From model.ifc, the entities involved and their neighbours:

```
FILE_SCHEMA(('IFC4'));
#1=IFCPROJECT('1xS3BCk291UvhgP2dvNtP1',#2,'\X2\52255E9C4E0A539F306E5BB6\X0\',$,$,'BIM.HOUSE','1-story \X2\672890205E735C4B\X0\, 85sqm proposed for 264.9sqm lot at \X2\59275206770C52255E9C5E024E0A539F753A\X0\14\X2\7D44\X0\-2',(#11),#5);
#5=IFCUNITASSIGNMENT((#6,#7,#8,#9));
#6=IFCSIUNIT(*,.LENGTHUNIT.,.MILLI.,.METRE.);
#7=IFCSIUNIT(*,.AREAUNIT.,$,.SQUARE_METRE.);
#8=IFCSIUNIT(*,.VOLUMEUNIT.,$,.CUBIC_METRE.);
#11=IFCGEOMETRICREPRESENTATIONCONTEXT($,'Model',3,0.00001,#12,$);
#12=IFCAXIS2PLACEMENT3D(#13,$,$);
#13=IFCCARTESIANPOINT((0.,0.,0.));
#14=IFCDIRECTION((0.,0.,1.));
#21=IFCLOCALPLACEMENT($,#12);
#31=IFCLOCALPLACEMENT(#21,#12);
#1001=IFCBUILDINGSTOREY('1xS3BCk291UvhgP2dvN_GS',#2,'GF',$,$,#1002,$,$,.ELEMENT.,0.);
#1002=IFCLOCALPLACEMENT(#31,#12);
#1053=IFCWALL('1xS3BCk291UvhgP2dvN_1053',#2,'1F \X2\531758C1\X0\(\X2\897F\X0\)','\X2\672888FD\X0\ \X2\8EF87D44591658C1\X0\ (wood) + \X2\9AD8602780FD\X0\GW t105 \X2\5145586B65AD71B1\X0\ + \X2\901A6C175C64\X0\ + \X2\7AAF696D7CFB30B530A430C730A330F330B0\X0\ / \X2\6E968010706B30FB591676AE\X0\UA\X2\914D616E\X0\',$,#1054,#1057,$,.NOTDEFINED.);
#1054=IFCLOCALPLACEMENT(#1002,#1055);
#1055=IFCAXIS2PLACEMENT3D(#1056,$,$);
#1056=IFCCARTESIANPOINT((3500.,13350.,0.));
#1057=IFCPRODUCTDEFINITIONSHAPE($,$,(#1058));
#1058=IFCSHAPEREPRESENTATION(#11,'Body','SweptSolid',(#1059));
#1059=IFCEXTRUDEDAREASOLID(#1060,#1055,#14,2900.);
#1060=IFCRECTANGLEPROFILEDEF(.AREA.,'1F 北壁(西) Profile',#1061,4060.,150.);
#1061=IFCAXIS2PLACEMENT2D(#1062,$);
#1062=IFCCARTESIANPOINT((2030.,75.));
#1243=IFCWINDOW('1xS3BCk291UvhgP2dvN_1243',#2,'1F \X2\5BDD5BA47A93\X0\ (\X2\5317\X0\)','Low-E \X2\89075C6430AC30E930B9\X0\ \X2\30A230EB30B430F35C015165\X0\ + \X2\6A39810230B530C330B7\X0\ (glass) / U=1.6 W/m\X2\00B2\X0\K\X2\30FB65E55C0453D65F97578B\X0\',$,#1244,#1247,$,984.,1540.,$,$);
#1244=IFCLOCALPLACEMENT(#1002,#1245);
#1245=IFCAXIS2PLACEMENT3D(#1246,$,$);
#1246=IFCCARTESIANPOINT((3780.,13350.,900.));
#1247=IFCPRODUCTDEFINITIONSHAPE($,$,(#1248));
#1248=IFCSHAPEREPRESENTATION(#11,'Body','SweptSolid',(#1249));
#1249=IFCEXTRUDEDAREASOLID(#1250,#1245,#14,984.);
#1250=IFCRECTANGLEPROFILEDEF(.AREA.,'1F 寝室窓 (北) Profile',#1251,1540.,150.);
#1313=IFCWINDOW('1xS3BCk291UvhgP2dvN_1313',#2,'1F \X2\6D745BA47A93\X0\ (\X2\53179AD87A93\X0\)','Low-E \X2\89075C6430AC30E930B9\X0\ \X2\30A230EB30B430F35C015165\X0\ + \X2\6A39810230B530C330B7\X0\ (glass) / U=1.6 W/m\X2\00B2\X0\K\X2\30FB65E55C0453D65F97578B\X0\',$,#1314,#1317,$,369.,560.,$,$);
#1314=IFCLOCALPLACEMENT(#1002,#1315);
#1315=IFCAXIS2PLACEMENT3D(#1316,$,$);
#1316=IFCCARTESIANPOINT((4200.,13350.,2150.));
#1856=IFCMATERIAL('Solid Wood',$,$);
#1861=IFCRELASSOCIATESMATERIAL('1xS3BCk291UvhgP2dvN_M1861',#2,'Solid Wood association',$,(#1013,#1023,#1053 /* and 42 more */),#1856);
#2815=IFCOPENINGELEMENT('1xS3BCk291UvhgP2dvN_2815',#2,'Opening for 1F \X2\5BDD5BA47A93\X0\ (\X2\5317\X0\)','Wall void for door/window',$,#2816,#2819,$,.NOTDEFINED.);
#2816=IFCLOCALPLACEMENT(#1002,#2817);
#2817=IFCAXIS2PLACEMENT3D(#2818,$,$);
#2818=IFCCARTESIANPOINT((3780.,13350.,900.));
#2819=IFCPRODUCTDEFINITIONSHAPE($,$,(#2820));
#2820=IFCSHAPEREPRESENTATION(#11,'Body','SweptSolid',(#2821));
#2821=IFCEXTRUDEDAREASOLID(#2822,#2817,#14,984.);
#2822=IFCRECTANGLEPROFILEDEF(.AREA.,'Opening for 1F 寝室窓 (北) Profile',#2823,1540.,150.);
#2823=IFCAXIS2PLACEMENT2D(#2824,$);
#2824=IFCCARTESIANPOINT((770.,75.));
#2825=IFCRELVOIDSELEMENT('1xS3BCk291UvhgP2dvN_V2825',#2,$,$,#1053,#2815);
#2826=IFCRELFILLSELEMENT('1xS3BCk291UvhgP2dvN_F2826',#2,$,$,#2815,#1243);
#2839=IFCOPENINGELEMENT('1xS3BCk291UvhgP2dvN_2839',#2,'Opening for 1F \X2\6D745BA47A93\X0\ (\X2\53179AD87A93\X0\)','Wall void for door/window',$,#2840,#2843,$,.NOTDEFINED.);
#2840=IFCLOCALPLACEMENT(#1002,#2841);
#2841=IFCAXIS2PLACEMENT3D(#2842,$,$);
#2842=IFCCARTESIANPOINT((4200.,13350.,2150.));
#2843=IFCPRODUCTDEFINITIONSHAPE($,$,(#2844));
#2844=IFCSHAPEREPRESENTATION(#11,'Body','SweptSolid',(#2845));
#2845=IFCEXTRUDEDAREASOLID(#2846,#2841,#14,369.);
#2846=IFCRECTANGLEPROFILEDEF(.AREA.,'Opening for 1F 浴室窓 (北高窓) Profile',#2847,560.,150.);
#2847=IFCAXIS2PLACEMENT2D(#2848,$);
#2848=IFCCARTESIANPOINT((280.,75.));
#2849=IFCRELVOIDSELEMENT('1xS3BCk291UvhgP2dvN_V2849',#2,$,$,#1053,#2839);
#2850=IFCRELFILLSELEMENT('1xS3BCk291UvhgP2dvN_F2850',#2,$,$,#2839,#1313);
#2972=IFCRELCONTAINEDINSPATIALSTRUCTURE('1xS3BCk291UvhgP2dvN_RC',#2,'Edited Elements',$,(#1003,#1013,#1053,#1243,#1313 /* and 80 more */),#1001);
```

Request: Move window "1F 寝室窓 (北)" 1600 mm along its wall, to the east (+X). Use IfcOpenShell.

```python
import ifcopenshell
import ifcopenshell.api.geometry
import ifcopenshell.util.placement

model = ifcopenshell.open("model.ifc")

window = model.by_guid("1xS3BCk291UvhgP2dvN_1243")
opening = window.FillsVoids[0].RelatingOpeningElement
wall = opening.VoidsElements[0].RelatingBuildingElement

wall_matrix = ifcopenshell.util.placement.get_local_placement(wall.ObjectPlacement)
shift = wall_matrix[:3, 0] * 1600.0
before = ifcopenshell.util.placement.get_local_placement(window.ObjectPlacement)[:3, 3].copy()

# The window is not placed relative to its opening, so move both.
for product in (opening, window):
    matrix = ifcopenshell.util.placement.get_local_placement(product.ObjectPlacement)
    matrix[:3, 3] += shift
    ifcopenshell.api.geometry.edit_object_placement(model, product=product, matrix=matrix, is_si=False)

after = ifcopenshell.util.placement.get_local_placement(window.ObjectPlacement)[:3, 3]
print("window moved by", (after - before).round(3) + 0.0)

model.write("model_edited.ifc")
```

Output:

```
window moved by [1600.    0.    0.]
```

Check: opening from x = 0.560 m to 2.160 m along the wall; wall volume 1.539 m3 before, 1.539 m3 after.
